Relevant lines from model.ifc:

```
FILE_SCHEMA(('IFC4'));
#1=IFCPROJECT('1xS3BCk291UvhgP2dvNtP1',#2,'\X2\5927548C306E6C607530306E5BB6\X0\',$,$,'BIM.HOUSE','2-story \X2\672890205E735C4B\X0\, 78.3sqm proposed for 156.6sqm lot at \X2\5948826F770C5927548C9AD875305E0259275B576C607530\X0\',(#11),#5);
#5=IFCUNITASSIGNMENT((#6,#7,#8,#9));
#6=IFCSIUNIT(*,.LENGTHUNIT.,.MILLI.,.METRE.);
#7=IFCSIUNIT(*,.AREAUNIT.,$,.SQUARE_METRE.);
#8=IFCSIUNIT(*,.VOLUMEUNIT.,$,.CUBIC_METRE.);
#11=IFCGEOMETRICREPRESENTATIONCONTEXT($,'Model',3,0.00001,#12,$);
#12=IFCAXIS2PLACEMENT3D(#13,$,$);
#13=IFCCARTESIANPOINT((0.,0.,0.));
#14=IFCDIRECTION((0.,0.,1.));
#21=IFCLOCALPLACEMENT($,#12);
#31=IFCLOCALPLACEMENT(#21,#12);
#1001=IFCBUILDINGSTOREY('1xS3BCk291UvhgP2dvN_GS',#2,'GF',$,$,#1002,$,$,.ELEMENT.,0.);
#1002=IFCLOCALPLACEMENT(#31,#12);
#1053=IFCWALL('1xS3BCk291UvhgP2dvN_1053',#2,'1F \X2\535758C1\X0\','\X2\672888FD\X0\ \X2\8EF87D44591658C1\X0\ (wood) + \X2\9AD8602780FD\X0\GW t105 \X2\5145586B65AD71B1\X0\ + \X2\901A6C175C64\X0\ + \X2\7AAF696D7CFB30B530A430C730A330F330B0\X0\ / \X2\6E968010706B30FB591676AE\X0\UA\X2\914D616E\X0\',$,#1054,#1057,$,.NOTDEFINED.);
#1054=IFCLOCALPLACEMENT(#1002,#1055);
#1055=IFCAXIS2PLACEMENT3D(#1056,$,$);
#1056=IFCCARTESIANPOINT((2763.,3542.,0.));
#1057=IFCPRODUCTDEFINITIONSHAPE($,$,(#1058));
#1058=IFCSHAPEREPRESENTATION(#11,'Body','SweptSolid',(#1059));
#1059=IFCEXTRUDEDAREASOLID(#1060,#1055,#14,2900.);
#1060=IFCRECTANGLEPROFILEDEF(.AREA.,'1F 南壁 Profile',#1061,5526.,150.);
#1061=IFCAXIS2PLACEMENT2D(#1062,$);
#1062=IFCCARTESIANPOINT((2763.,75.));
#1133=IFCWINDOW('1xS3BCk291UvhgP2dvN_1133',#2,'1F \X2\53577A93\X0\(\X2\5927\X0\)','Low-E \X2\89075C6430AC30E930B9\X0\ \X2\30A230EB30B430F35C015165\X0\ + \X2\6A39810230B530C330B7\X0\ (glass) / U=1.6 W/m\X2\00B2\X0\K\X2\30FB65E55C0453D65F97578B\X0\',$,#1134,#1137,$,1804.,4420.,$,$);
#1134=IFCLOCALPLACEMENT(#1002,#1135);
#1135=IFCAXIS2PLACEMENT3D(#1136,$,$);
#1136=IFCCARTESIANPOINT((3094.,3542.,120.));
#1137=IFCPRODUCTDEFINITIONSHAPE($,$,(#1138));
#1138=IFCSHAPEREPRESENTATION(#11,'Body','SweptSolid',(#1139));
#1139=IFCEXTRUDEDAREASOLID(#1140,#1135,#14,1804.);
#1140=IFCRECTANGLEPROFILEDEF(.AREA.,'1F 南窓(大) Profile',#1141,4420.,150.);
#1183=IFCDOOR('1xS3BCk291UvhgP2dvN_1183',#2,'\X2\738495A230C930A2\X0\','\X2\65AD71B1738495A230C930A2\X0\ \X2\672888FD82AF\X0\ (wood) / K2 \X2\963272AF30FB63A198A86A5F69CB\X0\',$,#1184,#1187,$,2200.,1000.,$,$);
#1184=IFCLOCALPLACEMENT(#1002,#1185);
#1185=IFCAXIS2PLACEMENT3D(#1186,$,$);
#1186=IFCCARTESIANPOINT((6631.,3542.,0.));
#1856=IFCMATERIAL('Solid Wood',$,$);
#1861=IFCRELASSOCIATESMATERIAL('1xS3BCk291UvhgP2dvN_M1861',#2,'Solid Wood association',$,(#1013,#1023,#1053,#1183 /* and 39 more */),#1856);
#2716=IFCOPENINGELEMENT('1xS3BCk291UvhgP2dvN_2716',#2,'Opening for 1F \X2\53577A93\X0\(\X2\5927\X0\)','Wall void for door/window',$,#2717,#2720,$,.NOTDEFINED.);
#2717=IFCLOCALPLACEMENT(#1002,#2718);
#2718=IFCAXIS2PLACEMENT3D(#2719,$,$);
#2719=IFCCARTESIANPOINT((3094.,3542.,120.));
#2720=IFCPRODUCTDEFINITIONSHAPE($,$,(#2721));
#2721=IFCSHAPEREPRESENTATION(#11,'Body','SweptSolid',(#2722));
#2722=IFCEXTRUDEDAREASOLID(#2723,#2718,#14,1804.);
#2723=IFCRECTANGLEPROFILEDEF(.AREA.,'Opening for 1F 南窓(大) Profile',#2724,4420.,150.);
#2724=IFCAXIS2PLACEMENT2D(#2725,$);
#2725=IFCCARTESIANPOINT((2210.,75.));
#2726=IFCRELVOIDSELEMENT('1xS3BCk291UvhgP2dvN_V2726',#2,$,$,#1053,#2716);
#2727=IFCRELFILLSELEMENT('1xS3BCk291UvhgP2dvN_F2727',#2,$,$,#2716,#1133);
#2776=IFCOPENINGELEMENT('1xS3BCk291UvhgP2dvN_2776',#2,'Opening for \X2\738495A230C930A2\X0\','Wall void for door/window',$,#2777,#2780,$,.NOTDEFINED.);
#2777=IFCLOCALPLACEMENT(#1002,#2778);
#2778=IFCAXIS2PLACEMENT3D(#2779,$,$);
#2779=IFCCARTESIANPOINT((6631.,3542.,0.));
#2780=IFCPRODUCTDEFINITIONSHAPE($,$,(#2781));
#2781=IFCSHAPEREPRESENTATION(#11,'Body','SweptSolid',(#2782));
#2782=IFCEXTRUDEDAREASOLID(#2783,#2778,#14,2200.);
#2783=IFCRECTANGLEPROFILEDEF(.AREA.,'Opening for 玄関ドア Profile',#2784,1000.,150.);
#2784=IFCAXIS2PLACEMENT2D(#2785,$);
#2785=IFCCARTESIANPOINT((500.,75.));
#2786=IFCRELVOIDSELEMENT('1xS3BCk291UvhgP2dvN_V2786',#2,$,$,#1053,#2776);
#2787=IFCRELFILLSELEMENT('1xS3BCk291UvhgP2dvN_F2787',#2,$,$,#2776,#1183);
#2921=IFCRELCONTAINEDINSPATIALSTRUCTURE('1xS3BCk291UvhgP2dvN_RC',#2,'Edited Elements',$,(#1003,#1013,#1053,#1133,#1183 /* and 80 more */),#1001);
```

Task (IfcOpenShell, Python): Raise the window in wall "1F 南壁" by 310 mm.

```python
import numpy as np
import ifcopenshell
import ifcopenshell.api.geometry
import ifcopenshell.util.placement
import ifcopenshell.util.unit

model = ifcopenshell.open("model.ifc")
unit_scale = ifcopenshell.util.unit.calculate_unit_scale(model)

window = model.by_guid("1xS3BCk291UvhgP2dvN_1133")
opening = window.FillsVoids[0].RelatingOpeningElement
dz = 0.31 / unit_scale

shift = np.array([0.0, 0.0, dz])
# The window is not placed relative to its opening, so move both.
for product in (opening, window):
    matrix = ifcopenshell.util.placement.get_local_placement(product.ObjectPlacement)
    matrix[:3, 3] += shift
    ifcopenshell.api.geometry.edit_object_placement(model, product=product, matrix=matrix, is_si=False)

print(f"moved by {dz * unit_scale:+.3f} m")

model.write("model_edited.ifc")
```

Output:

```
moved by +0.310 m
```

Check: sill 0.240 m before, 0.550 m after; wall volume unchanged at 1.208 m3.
